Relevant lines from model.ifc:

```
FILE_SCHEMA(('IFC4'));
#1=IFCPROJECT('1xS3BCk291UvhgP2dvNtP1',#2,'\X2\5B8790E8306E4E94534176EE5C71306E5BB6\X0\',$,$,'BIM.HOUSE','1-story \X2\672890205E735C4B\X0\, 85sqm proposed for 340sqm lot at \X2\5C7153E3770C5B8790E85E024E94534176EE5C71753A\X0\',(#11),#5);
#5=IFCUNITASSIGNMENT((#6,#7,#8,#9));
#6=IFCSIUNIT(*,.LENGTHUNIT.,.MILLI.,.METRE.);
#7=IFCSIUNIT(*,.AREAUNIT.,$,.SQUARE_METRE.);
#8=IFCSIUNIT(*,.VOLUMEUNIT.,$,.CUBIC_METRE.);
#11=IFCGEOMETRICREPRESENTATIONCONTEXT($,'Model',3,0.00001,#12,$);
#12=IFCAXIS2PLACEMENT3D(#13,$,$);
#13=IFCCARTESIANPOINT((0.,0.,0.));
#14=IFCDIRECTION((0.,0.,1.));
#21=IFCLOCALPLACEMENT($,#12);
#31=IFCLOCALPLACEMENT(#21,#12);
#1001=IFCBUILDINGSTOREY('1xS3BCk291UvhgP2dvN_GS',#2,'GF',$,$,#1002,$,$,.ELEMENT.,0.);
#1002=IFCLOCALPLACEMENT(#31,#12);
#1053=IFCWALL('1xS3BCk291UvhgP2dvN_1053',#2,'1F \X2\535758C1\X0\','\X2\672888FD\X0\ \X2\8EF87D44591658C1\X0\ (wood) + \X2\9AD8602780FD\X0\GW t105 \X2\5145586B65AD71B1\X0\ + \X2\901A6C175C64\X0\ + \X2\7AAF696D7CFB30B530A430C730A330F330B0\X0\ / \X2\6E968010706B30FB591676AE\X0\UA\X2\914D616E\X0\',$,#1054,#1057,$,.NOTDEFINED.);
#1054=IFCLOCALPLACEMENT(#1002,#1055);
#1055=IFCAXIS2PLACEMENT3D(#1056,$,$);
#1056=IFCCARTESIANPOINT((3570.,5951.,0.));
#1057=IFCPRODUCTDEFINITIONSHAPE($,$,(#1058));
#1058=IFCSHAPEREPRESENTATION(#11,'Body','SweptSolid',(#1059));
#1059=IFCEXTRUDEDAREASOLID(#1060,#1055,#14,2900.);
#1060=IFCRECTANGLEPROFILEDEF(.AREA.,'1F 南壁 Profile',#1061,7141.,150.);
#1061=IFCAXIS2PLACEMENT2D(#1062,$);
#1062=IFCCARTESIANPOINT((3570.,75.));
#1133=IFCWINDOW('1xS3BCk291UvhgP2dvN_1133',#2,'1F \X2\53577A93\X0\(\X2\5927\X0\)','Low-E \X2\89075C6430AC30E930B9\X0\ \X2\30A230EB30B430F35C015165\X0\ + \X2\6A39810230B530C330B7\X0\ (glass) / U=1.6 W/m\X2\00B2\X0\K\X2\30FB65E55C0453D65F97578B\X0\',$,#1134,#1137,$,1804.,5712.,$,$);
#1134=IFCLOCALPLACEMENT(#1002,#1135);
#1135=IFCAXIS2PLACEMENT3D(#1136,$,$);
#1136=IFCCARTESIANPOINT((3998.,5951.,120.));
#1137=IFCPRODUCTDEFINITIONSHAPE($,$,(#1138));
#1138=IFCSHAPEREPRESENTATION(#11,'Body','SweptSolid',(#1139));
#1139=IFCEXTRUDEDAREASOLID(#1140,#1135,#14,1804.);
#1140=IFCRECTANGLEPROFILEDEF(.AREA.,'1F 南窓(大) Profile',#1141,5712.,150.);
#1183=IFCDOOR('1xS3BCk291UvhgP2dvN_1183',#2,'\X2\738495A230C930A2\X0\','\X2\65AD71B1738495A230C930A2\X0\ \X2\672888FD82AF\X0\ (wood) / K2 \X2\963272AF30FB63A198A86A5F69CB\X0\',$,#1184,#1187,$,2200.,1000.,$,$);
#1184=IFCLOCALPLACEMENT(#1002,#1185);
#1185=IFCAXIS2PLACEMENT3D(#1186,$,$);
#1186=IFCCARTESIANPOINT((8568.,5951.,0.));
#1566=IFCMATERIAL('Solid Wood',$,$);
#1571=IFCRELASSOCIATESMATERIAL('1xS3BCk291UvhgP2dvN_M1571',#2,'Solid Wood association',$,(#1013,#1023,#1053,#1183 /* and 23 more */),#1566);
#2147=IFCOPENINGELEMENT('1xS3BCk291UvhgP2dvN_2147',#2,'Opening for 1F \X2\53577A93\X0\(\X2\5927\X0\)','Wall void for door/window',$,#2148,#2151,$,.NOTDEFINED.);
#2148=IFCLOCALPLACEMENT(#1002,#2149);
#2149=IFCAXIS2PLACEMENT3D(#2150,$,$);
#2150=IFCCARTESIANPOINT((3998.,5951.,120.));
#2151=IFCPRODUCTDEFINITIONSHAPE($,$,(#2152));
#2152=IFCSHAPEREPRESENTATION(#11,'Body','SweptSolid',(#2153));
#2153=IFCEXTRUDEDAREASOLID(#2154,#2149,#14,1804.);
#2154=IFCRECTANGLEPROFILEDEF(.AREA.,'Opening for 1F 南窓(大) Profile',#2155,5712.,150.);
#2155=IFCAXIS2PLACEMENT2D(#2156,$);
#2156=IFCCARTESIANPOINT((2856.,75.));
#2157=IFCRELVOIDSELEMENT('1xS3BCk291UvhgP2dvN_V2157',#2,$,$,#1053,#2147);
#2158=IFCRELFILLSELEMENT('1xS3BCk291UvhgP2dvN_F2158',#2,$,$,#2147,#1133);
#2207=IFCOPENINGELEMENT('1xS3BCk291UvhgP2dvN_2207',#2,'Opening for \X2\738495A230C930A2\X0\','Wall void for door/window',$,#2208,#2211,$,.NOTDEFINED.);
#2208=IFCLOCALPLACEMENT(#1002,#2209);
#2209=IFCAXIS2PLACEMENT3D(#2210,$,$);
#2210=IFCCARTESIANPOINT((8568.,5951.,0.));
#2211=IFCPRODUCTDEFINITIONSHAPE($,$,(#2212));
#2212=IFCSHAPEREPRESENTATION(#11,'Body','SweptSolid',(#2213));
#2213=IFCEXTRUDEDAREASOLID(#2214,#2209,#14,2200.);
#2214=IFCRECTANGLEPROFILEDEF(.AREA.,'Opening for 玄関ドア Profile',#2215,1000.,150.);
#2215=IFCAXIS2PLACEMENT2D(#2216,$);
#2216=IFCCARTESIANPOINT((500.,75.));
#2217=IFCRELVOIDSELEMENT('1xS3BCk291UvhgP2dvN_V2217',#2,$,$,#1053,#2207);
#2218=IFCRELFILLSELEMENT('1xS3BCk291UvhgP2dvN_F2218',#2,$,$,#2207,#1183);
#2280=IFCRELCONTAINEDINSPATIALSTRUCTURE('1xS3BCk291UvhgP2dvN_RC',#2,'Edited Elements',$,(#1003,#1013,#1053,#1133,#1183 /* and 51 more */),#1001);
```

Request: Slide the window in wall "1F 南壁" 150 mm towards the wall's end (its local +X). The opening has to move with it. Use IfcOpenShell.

```python
import ifcopenshell
import ifcopenshell.api.geometry
import ifcopenshell.util.placement

model = ifcopenshell.open("model.ifc")

window = model.by_id(1133)
opening = window.FillsVoids[0].RelatingOpeningElement
wall = opening.VoidsElements[0].RelatingBuildingElement

wall_matrix = ifcopenshell.util.placement.get_local_placement(wall.ObjectPlacement)
shift = wall_matrix[:3, 0] * 150.0
before = ifcopenshell.util.placement.get_local_placement(window.ObjectPlacement)[:3, 3].copy()

# The window is not placed relative to its opening, so move both.
for product in (opening, window):
    matrix = ifcopenshell.util.placement.get_local_placement(product.ObjectPlacement)
    matrix[:3, 3] += shift
    ifcopenshell.api.geometry.edit_object_placement(model, product=product, matrix=matrix, is_si=False)

after = ifcopenshell.util.placement.get_local_placement(window.ObjectPlacement)[:3, 3]
print("window moved by", (after - before).round(3) + 0.0)

model.write("model_rev.ifc")
```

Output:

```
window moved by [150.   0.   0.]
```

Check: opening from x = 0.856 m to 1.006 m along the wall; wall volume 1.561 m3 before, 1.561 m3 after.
